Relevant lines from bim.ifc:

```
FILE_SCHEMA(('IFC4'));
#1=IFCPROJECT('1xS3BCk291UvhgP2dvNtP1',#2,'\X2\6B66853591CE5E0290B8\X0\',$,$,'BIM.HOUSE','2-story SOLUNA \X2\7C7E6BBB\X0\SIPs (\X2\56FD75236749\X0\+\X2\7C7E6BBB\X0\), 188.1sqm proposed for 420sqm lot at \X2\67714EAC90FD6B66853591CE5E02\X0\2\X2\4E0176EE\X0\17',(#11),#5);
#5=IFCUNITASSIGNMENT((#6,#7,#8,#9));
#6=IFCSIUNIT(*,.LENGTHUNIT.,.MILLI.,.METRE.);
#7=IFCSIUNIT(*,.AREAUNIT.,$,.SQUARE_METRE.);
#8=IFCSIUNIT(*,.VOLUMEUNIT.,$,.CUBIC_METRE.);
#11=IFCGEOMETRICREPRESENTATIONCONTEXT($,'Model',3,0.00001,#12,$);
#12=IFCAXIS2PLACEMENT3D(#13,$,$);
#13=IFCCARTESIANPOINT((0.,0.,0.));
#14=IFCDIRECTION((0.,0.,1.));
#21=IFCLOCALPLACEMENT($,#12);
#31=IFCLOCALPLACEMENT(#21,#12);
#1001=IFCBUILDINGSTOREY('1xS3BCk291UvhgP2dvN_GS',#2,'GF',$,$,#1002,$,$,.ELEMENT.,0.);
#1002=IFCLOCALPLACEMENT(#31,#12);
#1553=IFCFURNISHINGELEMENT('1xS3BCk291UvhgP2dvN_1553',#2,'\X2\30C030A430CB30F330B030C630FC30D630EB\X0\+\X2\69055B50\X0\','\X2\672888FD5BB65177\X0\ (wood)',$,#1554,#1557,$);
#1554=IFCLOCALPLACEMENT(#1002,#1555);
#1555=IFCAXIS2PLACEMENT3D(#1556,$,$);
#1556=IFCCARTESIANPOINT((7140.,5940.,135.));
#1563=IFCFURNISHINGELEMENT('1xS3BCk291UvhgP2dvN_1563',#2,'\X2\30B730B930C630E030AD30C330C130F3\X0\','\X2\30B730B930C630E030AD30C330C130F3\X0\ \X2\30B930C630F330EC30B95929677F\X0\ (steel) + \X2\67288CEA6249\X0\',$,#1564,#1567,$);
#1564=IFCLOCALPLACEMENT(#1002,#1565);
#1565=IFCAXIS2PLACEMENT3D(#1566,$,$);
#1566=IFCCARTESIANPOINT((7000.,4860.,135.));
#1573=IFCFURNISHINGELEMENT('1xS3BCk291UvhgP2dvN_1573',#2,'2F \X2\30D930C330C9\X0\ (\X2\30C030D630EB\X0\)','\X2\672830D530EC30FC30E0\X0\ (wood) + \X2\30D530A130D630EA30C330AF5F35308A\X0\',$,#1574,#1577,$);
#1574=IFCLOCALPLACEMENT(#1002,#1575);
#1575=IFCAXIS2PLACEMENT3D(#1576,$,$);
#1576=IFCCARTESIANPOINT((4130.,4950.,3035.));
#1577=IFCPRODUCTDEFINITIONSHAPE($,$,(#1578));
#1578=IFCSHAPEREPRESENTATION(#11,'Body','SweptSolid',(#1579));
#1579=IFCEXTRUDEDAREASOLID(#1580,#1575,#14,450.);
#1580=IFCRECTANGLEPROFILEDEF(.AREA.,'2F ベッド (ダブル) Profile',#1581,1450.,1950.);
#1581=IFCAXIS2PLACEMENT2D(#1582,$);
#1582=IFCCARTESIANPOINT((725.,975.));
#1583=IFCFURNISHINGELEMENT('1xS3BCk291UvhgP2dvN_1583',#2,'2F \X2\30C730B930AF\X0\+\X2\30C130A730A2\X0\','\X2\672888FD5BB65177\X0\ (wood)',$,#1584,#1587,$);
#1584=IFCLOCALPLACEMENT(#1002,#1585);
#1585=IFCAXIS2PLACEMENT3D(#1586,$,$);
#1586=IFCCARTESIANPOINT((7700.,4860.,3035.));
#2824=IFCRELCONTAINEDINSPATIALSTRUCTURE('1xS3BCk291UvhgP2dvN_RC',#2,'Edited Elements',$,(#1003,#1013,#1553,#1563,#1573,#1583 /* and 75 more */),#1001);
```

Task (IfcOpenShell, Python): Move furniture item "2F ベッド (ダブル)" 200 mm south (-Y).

```python
import ifcopenshell
import ifcopenshell.api.geometry
import ifcopenshell.util.placement

model = ifcopenshell.open("bim.ifc")

item = model.by_id(1573)
matrix = ifcopenshell.util.placement.get_local_placement(item.ObjectPlacement)
matrix[1, 3] -= 200.0
ifcopenshell.api.geometry.edit_object_placement(model, product=item, matrix=matrix, is_si=False)

print(ifcopenshell.util.placement.get_local_placement(item.ObjectPlacement).round(3) + 0.0)

model.write("bim-out.ifc")
```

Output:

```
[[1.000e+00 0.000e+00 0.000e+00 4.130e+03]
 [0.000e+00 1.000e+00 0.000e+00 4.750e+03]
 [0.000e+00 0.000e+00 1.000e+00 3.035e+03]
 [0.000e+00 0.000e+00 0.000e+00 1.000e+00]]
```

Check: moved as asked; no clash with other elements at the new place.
